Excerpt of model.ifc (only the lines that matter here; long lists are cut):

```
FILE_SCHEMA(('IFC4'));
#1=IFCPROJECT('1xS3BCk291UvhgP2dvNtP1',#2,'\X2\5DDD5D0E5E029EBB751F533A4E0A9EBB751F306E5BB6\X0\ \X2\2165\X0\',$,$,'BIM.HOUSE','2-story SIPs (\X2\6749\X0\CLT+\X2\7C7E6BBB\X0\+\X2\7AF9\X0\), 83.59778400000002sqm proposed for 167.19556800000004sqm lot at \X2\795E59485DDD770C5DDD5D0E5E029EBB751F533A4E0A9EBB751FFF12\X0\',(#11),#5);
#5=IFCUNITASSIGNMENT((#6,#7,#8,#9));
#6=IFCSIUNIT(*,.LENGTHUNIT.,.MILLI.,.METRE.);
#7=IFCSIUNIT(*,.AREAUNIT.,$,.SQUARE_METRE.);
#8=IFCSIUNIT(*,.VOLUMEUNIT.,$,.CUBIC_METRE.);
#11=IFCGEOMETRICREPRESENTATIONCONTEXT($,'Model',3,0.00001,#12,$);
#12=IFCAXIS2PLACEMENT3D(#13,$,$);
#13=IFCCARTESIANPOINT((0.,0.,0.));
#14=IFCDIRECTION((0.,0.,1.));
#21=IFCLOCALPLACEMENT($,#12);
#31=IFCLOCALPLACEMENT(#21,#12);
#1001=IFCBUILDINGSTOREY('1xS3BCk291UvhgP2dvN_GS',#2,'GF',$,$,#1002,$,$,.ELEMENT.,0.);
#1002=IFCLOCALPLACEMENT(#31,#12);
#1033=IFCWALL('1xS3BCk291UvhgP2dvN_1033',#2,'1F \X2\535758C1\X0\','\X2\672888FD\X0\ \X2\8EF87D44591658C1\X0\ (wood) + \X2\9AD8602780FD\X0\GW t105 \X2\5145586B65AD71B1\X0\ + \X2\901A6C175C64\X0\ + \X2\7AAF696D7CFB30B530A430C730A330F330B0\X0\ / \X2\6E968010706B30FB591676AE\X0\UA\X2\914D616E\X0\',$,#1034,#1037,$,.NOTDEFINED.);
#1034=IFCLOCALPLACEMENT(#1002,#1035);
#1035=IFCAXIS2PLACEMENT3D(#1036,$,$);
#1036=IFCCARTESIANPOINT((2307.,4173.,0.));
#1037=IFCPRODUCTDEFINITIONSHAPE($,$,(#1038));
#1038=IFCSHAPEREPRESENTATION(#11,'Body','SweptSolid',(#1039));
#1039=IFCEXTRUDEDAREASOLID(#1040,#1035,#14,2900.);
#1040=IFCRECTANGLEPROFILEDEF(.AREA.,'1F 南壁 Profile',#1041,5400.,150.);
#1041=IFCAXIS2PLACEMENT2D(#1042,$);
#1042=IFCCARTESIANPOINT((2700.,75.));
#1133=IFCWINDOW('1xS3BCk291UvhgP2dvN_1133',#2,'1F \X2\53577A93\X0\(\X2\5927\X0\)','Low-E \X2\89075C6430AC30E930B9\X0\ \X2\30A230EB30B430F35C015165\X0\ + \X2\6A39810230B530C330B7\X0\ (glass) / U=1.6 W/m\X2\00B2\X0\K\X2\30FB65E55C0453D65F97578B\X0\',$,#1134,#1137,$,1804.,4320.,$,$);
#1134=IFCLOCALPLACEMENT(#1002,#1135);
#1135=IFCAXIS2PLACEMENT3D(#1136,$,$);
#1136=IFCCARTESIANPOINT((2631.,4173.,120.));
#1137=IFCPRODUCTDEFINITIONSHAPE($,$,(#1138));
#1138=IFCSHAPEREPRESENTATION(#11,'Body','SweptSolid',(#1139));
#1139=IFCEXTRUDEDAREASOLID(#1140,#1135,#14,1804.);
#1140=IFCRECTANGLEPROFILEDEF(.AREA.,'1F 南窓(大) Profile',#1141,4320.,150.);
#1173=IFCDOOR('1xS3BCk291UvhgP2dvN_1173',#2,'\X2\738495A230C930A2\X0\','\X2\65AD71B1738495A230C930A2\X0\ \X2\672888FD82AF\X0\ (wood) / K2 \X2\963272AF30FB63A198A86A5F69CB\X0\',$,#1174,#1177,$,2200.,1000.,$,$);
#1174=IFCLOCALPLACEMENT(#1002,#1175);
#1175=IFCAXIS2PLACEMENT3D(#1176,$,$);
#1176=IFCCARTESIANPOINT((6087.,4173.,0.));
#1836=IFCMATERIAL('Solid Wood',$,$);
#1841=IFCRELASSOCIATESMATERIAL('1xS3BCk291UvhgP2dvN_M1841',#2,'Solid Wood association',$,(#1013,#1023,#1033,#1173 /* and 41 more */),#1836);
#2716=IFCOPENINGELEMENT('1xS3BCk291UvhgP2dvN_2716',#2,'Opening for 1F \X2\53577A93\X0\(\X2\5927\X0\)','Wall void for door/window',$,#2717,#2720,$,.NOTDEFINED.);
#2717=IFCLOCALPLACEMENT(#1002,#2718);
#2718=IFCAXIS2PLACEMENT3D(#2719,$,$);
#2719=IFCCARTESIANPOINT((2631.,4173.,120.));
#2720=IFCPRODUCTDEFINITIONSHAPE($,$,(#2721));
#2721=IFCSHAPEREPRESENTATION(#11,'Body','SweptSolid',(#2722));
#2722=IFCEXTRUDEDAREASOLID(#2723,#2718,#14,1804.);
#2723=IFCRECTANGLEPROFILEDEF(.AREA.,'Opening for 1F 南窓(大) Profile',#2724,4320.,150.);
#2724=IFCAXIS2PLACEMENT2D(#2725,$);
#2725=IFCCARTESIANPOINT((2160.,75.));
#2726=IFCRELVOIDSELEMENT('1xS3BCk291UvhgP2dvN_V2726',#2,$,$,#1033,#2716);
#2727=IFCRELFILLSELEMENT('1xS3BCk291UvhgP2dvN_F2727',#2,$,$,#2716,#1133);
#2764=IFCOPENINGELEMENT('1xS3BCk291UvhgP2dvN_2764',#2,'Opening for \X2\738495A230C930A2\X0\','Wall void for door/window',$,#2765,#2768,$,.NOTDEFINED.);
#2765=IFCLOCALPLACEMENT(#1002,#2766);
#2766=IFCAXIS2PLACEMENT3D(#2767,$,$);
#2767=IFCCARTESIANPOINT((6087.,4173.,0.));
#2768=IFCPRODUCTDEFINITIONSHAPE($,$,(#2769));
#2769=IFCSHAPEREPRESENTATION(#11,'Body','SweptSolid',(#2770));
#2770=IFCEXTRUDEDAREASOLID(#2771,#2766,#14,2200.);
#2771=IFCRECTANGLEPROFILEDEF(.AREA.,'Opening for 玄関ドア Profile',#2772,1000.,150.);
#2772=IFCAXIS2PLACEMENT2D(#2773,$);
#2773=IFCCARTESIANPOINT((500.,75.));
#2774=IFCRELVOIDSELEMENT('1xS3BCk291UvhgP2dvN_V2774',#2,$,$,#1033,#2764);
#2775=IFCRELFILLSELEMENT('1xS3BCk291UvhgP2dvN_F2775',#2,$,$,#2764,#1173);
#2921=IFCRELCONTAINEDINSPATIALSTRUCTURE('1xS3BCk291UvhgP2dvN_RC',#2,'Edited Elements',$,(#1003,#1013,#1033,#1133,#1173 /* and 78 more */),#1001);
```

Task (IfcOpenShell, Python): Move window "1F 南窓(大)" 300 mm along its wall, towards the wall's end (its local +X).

```python
import ifcopenshell
import ifcopenshell.api.geometry
import ifcopenshell.util.placement
import ifcopenshell.util.unit

model = ifcopenshell.open("model.ifc")
unit_scale = ifcopenshell.util.unit.calculate_unit_scale(model)

window = model.by_id(1133)
opening = window.FillsVoids[0].RelatingOpeningElement
wall = opening.VoidsElements[0].RelatingBuildingElement

wall_matrix = ifcopenshell.util.placement.get_local_placement(wall.ObjectPlacement)
shift = wall_matrix[:3, 0] * 0.3 / unit_scale
before = ifcopenshell.util.placement.get_local_placement(window.ObjectPlacement)[:3, 3].copy()

# The window is not placed relative to its opening, so move both.
for product in (opening, window):
    matrix = ifcopenshell.util.placement.get_local_placement(product.ObjectPlacement)
    matrix[:3, 3] += shift
    ifcopenshell.api.geometry.edit_object_placement(model, product=product, matrix=matrix, is_si=False)

after = ifcopenshell.util.placement.get_local_placement(window.ObjectPlacement)[:3, 3]
print("window moved by", (after - before).round(3) + 0.0)

model.write("model_edited.ifc")
```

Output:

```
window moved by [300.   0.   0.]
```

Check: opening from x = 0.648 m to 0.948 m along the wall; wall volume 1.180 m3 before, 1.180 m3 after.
